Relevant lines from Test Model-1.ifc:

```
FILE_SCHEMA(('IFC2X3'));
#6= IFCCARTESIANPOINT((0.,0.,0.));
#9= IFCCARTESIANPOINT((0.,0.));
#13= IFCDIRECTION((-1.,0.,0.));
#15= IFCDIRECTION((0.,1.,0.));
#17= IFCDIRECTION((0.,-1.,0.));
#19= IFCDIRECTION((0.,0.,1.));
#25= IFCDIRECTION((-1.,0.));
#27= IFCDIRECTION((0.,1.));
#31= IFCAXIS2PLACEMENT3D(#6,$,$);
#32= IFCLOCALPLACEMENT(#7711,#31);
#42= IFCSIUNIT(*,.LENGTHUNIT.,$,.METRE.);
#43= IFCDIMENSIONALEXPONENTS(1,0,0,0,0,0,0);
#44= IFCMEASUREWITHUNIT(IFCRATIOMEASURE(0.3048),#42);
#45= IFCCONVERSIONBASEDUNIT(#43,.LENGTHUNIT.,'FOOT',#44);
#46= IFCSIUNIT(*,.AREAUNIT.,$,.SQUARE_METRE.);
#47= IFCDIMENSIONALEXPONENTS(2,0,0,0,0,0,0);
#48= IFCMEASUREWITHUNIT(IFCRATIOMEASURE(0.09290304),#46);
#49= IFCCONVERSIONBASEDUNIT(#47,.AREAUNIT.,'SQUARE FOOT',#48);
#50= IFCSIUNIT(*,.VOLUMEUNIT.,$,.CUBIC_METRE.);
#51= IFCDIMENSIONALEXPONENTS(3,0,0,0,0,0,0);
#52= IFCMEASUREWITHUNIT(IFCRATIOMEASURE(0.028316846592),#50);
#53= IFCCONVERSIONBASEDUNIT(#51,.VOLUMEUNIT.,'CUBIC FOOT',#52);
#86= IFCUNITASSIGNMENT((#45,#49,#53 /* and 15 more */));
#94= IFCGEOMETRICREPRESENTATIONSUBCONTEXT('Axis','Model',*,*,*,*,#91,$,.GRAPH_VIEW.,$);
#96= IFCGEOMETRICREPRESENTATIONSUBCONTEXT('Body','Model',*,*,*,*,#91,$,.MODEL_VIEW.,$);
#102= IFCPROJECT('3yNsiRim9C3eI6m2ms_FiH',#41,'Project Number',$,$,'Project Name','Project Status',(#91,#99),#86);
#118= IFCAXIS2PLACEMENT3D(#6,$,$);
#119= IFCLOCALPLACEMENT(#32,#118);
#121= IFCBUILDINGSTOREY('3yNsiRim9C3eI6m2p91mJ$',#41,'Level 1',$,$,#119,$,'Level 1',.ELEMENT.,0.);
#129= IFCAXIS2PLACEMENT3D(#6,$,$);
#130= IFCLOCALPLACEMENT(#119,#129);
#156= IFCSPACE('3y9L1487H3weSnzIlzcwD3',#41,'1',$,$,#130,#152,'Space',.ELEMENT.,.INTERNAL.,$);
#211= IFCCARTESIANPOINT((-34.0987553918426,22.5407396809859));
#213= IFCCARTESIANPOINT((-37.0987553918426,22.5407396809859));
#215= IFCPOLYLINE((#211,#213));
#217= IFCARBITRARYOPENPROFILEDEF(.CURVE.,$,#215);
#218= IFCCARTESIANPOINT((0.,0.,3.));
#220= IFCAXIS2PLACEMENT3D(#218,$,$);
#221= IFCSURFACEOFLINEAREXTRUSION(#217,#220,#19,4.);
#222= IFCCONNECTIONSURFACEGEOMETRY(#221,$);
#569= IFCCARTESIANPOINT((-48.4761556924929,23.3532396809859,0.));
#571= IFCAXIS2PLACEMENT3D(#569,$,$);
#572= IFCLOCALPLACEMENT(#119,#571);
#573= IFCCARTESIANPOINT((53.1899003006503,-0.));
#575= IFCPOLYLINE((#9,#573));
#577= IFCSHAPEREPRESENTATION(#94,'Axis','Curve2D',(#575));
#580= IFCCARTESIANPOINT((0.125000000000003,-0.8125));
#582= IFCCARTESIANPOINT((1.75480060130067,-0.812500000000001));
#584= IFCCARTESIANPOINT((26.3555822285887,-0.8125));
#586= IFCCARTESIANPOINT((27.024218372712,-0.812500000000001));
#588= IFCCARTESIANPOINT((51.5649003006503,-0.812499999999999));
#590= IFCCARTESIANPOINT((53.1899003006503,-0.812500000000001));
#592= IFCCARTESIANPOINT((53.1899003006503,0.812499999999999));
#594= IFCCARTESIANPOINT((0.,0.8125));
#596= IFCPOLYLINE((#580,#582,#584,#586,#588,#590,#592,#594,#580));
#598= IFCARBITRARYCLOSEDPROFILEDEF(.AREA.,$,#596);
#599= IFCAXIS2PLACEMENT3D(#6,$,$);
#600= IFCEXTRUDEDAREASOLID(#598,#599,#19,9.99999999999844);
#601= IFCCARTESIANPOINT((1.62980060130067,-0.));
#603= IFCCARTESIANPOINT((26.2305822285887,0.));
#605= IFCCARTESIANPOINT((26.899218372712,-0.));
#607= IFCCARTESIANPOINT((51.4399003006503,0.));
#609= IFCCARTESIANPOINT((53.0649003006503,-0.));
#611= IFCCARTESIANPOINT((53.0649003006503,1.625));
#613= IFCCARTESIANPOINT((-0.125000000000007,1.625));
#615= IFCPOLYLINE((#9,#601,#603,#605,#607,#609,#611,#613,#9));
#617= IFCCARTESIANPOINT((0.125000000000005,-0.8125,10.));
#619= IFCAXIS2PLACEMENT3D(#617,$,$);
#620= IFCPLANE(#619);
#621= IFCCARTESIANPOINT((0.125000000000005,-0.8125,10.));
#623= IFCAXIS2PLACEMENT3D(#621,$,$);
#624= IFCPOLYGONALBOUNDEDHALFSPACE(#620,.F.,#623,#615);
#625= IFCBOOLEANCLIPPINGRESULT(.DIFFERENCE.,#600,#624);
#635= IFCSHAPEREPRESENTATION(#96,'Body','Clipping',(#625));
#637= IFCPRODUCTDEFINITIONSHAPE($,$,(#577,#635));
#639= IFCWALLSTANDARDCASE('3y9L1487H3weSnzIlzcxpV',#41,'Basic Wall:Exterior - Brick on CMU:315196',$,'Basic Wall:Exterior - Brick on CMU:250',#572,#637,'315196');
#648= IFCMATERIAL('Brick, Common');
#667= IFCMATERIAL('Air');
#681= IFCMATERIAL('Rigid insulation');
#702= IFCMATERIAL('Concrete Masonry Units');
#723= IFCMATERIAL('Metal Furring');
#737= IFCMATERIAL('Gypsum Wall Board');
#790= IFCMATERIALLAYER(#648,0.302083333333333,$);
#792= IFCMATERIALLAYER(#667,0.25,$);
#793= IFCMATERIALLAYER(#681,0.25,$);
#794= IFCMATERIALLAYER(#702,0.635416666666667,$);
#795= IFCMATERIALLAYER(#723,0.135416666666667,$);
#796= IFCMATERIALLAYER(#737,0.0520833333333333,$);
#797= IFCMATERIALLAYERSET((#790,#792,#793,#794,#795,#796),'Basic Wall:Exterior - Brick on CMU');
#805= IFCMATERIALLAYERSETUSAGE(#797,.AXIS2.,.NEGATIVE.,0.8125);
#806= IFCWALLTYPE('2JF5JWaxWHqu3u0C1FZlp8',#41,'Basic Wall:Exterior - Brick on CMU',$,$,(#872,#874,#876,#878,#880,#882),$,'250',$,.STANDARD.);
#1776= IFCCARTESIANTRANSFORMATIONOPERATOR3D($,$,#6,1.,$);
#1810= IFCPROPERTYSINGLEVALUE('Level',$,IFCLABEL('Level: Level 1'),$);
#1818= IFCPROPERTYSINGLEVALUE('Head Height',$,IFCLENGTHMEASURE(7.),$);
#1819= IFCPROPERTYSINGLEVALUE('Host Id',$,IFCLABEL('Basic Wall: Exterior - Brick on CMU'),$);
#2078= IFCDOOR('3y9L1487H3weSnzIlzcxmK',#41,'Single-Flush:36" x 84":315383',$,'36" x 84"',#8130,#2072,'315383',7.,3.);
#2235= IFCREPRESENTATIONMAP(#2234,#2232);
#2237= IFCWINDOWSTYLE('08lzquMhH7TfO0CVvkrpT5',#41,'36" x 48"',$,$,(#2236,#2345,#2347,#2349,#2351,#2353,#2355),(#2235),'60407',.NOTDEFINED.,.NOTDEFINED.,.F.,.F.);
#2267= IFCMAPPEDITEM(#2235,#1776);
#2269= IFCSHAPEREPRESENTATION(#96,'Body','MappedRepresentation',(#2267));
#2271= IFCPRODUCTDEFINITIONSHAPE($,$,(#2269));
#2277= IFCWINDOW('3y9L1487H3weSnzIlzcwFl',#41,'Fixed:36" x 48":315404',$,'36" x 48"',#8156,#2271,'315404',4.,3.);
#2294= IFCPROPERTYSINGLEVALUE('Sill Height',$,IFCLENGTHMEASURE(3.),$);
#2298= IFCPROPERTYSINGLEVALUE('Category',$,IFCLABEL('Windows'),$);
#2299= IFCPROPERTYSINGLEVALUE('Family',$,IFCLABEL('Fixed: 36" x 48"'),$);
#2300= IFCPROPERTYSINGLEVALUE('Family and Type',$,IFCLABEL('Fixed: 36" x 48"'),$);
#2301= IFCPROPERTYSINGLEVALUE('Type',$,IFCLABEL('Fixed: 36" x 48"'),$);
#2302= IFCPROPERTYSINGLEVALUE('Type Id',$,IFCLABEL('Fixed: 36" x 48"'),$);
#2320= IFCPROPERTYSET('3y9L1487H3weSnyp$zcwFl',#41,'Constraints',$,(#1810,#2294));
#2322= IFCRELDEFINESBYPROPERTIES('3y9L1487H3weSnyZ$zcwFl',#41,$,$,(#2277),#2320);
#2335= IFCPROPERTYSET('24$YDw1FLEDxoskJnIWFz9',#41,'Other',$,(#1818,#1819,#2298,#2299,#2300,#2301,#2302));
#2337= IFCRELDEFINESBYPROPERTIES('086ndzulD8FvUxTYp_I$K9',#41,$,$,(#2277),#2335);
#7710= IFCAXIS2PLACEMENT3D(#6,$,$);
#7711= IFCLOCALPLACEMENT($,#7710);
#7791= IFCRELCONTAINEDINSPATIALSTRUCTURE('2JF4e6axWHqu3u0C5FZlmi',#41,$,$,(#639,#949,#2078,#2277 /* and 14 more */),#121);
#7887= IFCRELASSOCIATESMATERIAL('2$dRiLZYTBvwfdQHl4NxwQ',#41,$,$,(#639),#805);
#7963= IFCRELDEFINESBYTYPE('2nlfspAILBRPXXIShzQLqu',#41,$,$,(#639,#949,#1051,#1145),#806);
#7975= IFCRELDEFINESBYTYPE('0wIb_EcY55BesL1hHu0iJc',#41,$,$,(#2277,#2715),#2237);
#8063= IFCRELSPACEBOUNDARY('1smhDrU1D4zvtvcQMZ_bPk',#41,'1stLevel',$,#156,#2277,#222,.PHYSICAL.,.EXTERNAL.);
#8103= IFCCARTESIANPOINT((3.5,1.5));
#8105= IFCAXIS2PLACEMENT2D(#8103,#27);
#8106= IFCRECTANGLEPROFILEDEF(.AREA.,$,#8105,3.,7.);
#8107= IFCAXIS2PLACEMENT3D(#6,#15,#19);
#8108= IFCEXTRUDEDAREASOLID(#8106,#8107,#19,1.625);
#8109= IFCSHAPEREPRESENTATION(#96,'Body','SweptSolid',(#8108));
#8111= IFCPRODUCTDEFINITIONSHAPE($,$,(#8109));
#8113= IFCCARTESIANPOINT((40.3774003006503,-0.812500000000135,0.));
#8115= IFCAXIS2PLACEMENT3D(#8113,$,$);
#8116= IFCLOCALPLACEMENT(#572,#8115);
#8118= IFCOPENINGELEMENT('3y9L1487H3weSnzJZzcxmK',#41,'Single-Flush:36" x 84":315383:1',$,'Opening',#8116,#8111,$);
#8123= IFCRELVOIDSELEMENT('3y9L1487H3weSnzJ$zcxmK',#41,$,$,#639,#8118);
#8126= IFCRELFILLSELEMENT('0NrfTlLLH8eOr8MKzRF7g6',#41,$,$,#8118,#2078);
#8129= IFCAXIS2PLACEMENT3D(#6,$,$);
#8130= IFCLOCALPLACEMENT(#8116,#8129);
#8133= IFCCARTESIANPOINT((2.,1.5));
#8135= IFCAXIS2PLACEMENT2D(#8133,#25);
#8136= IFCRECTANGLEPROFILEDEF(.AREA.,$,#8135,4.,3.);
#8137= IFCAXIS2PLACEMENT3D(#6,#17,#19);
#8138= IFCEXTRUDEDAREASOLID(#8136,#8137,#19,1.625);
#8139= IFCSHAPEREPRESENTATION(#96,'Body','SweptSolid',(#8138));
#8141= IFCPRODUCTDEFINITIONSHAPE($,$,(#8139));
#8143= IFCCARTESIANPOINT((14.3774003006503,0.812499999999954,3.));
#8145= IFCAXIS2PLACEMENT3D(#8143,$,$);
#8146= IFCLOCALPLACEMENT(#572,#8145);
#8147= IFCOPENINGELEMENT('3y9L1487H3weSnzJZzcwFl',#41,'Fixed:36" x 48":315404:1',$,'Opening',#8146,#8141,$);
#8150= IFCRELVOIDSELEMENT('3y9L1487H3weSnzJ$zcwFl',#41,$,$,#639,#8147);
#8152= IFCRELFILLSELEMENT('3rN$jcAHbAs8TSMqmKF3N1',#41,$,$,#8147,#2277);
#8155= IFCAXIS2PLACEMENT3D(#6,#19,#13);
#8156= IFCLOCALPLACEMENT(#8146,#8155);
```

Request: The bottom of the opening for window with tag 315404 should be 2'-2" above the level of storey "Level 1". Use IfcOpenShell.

```python
import numpy as np
import ifcopenshell
import ifcopenshell.api.geometry
import ifcopenshell.api.pset
import ifcopenshell.geom
import ifcopenshell.util.element
import ifcopenshell.util.placement
import ifcopenshell.util.shape
import ifcopenshell.util.unit

model = ifcopenshell.open("Test Model-1.ifc")
unit_scale = ifcopenshell.util.unit.calculate_unit_scale(model)

window = model.by_guid("3y9L1487H3weSnzIlzcwFl")
opening = window.FillsVoids[0].RelatingOpeningElement
storey = ifcopenshell.util.element.get_container(window, ifc_class="IfcBuildingStorey")
level = ifcopenshell.util.placement.get_local_placement(storey.ObjectPlacement)[2, 3]

# The opening's origin need not be at the sill, so measure its lowest point.
shape = ifcopenshell.geom.create_shape(ifcopenshell.geom.settings(), opening)
bottom = ifcopenshell.util.shape.get_shape_bottom_elevation(shape, shape.geometry) / unit_scale
dz = level + 26 * 0.0254 / unit_scale - bottom

shift = np.array([0.0, 0.0, dz])
# The window is placed relative to its opening, so it follows when the opening moves.
matrix = ifcopenshell.util.placement.get_local_placement(opening.ObjectPlacement)
matrix[:3, 3] += shift
ifcopenshell.api.geometry.edit_object_placement(
    model, product=opening, matrix=matrix, is_si=False, should_transform_children=True
)

# Space boundary surfaces are stored in each space's coordinates; move them too.
for rel in window.ProvidesBoundaries:
    if not rel.ConnectionGeometry:
        continue
    surface = rel.ConnectionGeometry.SurfaceOnRelatingElement
    space_matrix = ifcopenshell.util.placement.get_local_placement(rel.RelatingSpace.ObjectPlacement)
    point = np.array(surface.Position.Location.Coordinates) + space_matrix[:3, :3].T @ shift
    surface.Position = model.createIfcAxis2Placement3D(
        model.createIfcCartesianPoint(point.tolist()), surface.Position.Axis, surface.Position.RefDirection
    )

# Keep the stored heights in step.
pset = model.by_id(ifcopenshell.util.element.get_pset(window, "Constraints", should_inherit=False)["id"])
ifcopenshell.api.pset.edit_pset(model, pset=pset, properties={
    "Sill Height": model.create_entity("IfcLengthMeasure", ifcopenshell.util.element.get_pset(window, "Constraints", "Sill Height") + dz),
})
pset = model.by_id(ifcopenshell.util.element.get_pset(window, "Other", should_inherit=False)["id"])
ifcopenshell.api.pset.edit_pset(model, pset=pset, properties={
    "Head Height": model.create_entity("IfcLengthMeasure", ifcopenshell.util.element.get_pset(window, "Other", "Head Height") + dz),
})

print(f"moved by {dz * unit_scale:+.3f} m")

model.write("Test Model-1_updated.ifc")
```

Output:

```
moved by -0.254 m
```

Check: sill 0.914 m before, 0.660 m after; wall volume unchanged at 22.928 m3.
